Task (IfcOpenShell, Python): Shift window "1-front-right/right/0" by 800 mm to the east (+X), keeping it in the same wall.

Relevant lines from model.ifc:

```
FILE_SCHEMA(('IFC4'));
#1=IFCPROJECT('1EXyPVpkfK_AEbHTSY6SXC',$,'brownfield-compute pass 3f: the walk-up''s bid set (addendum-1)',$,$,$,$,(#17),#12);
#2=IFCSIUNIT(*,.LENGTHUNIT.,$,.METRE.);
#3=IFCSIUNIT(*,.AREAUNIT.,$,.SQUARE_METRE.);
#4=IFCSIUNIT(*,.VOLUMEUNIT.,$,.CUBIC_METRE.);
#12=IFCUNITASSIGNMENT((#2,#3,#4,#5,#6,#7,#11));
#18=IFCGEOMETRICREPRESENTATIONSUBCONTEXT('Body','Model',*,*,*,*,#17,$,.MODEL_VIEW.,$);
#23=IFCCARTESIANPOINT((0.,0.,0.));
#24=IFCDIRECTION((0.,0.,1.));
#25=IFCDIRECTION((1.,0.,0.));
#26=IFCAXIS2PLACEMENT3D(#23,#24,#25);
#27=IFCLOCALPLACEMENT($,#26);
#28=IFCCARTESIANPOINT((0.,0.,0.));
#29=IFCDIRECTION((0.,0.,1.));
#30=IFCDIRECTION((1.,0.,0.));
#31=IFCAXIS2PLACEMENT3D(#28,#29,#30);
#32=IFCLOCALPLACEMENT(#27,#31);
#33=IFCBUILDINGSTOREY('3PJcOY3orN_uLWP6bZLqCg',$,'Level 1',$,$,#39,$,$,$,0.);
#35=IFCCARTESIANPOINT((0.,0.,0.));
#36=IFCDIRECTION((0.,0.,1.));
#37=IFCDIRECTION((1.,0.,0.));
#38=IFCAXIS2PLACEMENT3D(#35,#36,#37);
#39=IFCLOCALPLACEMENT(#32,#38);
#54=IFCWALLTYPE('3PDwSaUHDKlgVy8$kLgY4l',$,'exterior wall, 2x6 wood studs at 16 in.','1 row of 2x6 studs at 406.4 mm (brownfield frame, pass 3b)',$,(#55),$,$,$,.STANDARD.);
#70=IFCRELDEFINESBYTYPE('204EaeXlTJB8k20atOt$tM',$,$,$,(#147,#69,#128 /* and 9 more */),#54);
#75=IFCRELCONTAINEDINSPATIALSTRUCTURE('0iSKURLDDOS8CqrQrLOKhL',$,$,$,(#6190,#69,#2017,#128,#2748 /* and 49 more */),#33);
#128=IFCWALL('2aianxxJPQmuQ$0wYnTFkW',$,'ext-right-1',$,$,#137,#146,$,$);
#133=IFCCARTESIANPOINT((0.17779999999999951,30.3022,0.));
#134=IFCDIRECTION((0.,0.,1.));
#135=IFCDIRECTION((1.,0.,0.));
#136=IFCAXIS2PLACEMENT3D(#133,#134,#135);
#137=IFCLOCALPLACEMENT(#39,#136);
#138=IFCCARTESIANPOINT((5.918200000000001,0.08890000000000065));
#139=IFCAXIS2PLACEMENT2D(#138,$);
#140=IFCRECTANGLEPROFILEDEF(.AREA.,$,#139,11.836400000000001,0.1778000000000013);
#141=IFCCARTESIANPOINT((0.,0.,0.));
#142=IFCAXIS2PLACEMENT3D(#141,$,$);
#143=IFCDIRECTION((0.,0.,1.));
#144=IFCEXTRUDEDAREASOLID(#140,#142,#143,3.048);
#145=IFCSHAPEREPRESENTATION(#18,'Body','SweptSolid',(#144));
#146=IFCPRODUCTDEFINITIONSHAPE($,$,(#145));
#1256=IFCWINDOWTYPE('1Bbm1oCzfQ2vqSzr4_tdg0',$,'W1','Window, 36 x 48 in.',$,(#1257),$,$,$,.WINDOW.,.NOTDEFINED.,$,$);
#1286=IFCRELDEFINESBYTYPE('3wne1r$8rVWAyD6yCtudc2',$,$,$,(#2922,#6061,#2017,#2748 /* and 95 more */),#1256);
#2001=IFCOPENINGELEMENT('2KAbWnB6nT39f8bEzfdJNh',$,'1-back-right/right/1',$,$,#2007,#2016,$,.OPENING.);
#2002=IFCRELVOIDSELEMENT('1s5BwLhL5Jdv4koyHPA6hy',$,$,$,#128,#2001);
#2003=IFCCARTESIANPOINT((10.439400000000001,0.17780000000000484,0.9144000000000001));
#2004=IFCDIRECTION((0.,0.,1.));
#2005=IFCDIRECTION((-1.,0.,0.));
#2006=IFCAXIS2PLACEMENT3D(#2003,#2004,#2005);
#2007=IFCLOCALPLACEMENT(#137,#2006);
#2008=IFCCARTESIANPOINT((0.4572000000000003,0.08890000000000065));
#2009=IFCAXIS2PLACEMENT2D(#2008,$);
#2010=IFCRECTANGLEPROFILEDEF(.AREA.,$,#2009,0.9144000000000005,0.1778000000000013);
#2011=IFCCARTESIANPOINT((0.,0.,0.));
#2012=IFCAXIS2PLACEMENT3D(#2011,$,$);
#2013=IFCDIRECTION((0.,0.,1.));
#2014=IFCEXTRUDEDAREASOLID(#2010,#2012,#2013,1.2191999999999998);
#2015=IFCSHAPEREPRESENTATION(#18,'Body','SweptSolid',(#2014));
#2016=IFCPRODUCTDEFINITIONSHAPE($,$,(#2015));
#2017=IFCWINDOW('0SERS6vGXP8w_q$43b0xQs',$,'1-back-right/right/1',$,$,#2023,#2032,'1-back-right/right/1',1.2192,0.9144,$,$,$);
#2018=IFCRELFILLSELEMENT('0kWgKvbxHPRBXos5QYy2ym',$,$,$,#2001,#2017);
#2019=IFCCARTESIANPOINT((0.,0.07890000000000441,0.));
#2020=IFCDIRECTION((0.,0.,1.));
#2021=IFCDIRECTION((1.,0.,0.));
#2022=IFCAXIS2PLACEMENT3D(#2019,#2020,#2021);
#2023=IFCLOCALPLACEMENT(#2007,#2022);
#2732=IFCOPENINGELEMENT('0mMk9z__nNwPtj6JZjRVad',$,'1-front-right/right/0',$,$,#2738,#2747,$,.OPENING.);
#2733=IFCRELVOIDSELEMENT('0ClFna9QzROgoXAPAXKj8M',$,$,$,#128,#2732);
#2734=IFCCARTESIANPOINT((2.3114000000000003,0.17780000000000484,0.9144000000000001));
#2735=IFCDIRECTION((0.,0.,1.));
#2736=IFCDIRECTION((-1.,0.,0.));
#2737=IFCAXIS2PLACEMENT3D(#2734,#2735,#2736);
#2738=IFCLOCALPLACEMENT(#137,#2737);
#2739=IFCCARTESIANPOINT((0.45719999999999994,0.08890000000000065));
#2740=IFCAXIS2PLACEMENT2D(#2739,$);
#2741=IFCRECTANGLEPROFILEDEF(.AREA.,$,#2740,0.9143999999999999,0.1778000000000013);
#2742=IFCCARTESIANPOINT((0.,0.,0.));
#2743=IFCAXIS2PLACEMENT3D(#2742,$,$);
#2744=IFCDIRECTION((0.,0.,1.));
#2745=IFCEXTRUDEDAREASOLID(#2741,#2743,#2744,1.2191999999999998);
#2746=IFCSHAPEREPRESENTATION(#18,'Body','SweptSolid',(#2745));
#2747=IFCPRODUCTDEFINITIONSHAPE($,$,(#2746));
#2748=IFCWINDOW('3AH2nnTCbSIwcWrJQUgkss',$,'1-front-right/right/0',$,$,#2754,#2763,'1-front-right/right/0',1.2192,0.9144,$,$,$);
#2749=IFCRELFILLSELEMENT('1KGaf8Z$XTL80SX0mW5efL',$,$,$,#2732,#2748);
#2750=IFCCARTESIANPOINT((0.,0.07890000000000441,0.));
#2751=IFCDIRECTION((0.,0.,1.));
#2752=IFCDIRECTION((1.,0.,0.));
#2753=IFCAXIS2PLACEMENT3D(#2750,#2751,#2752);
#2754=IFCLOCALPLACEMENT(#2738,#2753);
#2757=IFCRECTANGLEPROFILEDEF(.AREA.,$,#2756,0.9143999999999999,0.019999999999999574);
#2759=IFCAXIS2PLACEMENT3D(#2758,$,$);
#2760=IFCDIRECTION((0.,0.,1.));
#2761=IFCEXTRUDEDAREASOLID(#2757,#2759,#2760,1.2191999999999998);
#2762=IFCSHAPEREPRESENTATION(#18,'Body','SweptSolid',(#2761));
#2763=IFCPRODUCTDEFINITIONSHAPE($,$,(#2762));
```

```python
import ifcopenshell
import ifcopenshell.api.geometry
import ifcopenshell.util.placement

model = ifcopenshell.open("model.ifc")

window = model.by_id(2748)
opening = window.FillsVoids[0].RelatingOpeningElement
wall = opening.VoidsElements[0].RelatingBuildingElement

wall_matrix = ifcopenshell.util.placement.get_local_placement(wall.ObjectPlacement)
shift = wall_matrix[:3, 0] * 0.8
before = ifcopenshell.util.placement.get_local_placement(window.ObjectPlacement)[:3, 3].copy()

# The window is placed relative to its opening, so it follows when the opening moves.
matrix = ifcopenshell.util.placement.get_local_placement(opening.ObjectPlacement)
matrix[:3, 3] += shift
ifcopenshell.api.geometry.edit_object_placement(
    model, product=opening, matrix=matrix, is_si=False, should_transform_children=True
)

after = ifcopenshell.util.placement.get_local_placement(window.ObjectPlacement)[:3, 3]
print("window moved by", (after - before).round(3) + 0.0)

model.write("model_edited.ifc")
```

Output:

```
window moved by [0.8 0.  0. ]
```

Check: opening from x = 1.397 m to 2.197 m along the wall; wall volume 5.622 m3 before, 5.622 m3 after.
